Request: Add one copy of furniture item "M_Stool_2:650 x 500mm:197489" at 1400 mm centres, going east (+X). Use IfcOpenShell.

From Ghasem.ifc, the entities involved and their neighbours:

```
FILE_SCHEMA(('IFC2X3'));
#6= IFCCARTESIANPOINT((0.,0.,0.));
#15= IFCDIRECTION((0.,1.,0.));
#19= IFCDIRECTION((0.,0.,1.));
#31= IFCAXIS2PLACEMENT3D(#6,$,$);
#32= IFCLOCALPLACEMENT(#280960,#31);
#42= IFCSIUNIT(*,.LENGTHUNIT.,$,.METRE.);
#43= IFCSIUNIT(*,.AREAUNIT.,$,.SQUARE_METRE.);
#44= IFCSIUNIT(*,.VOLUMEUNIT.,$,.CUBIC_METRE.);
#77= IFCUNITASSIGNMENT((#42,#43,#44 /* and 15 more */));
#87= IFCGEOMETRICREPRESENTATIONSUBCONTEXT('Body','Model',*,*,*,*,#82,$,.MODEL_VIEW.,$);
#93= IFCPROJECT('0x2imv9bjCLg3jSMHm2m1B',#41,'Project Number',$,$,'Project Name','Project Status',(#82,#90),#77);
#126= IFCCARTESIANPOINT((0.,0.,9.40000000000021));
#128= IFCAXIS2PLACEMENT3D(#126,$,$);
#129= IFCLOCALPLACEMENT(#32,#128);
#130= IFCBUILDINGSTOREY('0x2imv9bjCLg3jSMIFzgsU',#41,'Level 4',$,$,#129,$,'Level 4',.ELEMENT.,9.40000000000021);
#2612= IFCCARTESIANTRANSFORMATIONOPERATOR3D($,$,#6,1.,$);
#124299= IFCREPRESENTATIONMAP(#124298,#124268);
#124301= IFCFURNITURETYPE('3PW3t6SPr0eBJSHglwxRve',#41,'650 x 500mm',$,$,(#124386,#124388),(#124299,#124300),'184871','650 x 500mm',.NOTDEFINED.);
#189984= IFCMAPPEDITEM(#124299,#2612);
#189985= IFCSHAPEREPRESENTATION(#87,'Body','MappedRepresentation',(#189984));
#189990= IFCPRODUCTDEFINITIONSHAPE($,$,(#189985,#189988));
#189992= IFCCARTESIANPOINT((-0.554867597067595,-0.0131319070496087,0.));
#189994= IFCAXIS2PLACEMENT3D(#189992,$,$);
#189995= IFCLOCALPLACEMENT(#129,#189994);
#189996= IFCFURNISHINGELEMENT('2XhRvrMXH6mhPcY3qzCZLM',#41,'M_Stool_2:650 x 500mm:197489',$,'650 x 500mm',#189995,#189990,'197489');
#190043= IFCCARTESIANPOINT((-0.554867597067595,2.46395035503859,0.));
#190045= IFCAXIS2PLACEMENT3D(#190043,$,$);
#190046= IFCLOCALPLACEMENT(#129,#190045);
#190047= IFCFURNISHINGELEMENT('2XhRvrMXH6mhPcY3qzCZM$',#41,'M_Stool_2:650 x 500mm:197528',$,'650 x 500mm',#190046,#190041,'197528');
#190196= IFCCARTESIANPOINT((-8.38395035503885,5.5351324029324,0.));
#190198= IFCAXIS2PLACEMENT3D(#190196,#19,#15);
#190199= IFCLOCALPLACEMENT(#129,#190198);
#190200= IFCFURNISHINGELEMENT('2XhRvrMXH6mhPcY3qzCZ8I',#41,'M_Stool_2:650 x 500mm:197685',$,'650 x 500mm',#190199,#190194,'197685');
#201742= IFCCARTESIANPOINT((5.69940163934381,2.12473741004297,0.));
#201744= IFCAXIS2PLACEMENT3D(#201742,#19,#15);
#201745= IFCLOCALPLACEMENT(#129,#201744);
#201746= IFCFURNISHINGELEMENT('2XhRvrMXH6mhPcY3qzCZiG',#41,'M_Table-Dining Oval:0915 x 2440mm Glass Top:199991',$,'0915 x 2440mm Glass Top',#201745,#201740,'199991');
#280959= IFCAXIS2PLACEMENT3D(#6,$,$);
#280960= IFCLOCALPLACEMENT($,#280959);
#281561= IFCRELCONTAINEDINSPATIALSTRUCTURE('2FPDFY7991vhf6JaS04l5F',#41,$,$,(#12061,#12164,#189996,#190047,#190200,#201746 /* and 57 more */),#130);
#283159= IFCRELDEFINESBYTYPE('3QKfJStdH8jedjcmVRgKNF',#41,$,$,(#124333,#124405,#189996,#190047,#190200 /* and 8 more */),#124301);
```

```python
import numpy as np
import ifcopenshell
import ifcopenshell.api.geometry
import ifcopenshell.api.root
import ifcopenshell.util.element
import ifcopenshell.util.placement
import ifcopenshell.util.unit

model = ifcopenshell.open("Ghasem.ifc")
unit_scale = ifcopenshell.util.unit.calculate_unit_scale(model)


def reuse_history(source, copy):
    """copy_class also copies each property set's owner history, people and application; keep the originals."""
    for rel in copy.IsDefinedBy:
        if rel.is_a("IfcRelDefinesByProperties") and (history := rel.RelatingPropertyDefinition.OwnerHistory):
            rel.RelatingPropertyDefinition.OwnerHistory = source.OwnerHistory
            ifcopenshell.util.element.remove_deep2(model, history)


source = model.by_guid("2XhRvrMXH6mhPcY3qzCZLM")
base = ifcopenshell.util.placement.get_local_placement(source.ObjectPlacement)
step = np.array([1.0, 0.0, 0.0]) * 1.4 / unit_scale

for i in range(1, 2):
    copy = ifcopenshell.api.root.copy_class(model, product=source)
    copy.Representation = ifcopenshell.util.element.copy_deep(
        model, source.Representation, exclude=["IfcGeometricRepresentationContext", "IfcRepresentationMap"]
    )
    copy.Name = "M_Stool_2:650 x 500mm"
    copy.Tag = None
    reuse_history(source, copy)
    matrix = base.copy()
    matrix[:3, 3] += i * step
    print("added at", matrix[:3, 3].round(3) + 0.0)
    ifcopenshell.api.geometry.edit_object_placement(model, product=copy, matrix=matrix, is_si=False)

model.write("Ghasem_v2.ifc")
```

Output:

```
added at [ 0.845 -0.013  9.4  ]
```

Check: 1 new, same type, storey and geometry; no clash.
